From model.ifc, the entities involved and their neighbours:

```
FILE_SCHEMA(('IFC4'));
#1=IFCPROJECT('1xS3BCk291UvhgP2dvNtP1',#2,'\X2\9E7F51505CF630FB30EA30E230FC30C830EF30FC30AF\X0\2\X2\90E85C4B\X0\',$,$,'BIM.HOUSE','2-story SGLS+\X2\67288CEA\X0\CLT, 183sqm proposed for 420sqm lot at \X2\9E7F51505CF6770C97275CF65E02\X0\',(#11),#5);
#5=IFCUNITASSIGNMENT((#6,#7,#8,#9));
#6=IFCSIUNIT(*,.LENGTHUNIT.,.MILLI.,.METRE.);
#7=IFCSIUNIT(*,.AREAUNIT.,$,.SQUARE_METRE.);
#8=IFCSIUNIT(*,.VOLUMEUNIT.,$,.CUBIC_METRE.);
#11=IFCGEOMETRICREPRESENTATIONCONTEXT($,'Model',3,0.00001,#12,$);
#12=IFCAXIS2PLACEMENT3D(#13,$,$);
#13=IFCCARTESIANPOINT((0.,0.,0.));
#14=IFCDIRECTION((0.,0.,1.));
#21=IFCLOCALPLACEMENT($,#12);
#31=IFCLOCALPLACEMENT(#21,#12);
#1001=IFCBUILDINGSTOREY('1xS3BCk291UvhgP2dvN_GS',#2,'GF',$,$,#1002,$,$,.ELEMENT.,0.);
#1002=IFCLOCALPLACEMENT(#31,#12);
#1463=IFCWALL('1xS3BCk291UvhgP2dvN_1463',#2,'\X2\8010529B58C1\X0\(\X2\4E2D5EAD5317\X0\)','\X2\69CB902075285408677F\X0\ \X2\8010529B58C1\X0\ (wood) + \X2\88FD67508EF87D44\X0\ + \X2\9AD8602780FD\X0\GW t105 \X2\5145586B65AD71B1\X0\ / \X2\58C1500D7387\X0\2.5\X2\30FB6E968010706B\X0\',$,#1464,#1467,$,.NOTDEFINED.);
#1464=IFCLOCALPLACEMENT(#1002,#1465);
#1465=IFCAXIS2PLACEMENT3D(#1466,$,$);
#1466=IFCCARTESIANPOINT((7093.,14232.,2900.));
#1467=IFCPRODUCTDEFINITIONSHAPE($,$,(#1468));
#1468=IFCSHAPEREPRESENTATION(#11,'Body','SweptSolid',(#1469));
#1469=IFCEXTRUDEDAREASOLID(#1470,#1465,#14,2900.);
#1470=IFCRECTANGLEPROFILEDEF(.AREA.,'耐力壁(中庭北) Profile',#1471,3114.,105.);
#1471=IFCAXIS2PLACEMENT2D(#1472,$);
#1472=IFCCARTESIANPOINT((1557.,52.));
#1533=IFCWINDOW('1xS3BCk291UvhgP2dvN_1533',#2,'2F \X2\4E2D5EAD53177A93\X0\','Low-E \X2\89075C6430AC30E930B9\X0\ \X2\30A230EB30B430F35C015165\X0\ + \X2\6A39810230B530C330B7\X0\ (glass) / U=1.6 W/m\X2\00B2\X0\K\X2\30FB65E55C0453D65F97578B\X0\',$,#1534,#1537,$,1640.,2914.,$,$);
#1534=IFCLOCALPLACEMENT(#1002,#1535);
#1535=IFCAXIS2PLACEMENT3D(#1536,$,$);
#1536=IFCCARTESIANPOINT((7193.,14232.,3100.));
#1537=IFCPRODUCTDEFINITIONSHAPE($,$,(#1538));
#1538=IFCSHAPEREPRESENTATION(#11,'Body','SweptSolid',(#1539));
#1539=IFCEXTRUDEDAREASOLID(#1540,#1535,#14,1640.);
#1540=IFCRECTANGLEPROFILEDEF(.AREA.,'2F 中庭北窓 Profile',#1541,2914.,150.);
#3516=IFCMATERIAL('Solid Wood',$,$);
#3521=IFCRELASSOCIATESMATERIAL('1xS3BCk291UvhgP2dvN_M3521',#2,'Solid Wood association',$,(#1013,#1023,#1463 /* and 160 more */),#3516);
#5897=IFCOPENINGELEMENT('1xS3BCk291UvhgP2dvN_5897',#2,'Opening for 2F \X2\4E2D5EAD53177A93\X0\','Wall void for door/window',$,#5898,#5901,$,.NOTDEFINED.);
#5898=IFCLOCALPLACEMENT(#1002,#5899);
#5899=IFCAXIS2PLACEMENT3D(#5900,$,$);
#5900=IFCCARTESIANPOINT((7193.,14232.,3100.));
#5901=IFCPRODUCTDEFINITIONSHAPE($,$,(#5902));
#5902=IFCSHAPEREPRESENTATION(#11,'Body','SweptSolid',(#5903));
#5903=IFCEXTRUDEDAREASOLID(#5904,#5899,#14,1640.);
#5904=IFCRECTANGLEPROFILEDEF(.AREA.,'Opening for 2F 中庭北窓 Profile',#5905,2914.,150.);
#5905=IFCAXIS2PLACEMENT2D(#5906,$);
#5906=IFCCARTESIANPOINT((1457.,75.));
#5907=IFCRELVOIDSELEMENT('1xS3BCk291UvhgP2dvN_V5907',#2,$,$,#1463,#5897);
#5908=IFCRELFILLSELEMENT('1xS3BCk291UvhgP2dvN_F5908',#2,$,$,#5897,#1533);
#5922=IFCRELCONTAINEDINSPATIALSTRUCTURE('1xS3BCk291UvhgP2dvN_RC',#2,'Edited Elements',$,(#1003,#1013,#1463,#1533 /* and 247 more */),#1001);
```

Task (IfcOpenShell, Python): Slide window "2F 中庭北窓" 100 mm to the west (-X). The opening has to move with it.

```python
import ifcopenshell
import ifcopenshell.api.geometry
import ifcopenshell.util.placement

model = ifcopenshell.open("model.ifc")

window = model.by_id(1533)
opening = window.FillsVoids[0].RelatingOpeningElement
wall = opening.VoidsElements[0].RelatingBuildingElement

wall_matrix = ifcopenshell.util.placement.get_local_placement(wall.ObjectPlacement)
shift = wall_matrix[:3, 0] * -100.0
before = ifcopenshell.util.placement.get_local_placement(window.ObjectPlacement)[:3, 3].copy()

# The window is not placed relative to its opening, so move both.
for product in (opening, window):
    matrix = ifcopenshell.util.placement.get_local_placement(product.ObjectPlacement)
    matrix[:3, 3] += shift
    ifcopenshell.api.geometry.edit_object_placement(model, product=product, matrix=matrix, is_si=False)

after = ifcopenshell.util.placement.get_local_placement(window.ObjectPlacement)[:3, 3]
print("window moved by", (after - before).round(3) + 0.0)

model.write("model_rev.ifc")
```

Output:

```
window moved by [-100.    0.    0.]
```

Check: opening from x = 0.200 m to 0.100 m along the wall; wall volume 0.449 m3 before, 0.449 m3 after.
